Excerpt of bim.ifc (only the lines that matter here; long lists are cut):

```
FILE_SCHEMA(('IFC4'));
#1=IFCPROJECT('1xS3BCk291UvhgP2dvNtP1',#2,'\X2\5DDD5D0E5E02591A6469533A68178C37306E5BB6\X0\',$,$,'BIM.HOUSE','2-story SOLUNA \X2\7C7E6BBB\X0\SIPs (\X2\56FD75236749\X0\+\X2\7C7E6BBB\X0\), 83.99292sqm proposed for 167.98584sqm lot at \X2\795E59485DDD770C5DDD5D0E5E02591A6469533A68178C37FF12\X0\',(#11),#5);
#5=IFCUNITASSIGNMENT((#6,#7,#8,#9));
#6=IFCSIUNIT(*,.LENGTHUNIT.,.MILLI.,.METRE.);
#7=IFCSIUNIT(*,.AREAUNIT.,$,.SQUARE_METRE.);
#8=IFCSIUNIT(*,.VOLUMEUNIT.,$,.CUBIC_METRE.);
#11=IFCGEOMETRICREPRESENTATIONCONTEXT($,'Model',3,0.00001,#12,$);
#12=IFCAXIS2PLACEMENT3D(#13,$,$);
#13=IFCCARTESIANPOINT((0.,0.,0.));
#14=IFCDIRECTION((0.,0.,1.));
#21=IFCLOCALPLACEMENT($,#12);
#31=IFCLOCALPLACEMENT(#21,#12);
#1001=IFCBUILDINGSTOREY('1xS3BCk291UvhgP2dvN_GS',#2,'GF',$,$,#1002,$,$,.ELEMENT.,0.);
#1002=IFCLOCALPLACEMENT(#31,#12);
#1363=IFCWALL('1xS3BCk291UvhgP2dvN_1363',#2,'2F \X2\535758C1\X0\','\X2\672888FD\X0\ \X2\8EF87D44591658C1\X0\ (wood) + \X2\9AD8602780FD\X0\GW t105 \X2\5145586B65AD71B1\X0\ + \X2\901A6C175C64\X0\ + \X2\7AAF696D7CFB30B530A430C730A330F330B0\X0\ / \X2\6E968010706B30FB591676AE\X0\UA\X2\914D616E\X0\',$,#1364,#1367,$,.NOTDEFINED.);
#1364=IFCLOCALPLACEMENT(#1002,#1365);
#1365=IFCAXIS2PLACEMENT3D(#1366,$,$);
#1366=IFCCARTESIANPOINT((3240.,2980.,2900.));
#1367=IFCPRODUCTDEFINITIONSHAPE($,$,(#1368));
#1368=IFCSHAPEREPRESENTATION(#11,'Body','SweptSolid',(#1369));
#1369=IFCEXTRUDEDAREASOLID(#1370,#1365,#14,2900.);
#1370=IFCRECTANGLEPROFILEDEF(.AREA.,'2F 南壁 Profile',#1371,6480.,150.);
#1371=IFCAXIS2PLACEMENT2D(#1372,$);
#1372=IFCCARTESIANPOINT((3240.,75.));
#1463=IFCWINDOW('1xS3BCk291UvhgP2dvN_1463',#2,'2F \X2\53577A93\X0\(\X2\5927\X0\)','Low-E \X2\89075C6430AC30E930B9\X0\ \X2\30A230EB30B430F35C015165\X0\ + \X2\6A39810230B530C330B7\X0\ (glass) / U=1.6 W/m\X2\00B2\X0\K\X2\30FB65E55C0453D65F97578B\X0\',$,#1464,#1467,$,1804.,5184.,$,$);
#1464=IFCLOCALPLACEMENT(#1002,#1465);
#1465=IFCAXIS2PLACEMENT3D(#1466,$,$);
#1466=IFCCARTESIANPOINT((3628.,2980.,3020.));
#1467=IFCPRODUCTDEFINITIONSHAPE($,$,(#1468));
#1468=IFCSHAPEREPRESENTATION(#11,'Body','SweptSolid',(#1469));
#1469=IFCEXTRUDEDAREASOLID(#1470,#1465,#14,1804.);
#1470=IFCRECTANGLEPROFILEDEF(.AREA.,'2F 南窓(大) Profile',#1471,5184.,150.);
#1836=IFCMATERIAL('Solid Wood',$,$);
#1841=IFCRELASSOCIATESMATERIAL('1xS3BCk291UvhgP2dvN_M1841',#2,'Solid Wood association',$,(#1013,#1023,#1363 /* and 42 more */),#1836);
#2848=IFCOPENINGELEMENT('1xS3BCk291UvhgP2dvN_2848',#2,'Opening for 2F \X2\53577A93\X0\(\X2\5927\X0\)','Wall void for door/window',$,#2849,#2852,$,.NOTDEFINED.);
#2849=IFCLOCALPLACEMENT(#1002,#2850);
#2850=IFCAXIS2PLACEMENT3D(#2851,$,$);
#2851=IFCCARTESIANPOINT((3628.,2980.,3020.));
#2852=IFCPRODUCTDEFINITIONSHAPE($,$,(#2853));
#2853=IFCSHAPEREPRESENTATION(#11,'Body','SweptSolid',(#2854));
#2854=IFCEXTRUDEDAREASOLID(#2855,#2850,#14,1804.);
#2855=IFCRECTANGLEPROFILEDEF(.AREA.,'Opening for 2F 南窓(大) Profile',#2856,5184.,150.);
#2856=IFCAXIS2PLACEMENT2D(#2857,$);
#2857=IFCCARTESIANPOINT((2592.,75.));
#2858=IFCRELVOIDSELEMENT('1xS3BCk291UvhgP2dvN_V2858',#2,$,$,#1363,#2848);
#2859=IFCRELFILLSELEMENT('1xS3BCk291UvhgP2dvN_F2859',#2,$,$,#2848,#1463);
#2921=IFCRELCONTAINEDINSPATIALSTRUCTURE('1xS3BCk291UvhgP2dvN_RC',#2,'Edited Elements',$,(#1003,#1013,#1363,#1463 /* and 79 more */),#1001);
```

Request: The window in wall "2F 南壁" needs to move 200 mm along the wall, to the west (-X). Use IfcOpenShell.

```python
import ifcopenshell
import ifcopenshell.api.geometry
import ifcopenshell.util.placement

model = ifcopenshell.open("bim.ifc")

window = model.by_guid("1xS3BCk291UvhgP2dvN_1463")
opening = window.FillsVoids[0].RelatingOpeningElement
wall = opening.VoidsElements[0].RelatingBuildingElement

wall_matrix = ifcopenshell.util.placement.get_local_placement(wall.ObjectPlacement)
shift = wall_matrix[:3, 0] * -200.0
before = ifcopenshell.util.placement.get_local_placement(window.ObjectPlacement)[:3, 3].copy()

# The window is not placed relative to its opening, so move both.
for product in (opening, window):
    matrix = ifcopenshell.util.placement.get_local_placement(product.ObjectPlacement)
    matrix[:3, 3] += shift
    ifcopenshell.api.geometry.edit_object_placement(model, product=product, matrix=matrix, is_si=False)

after = ifcopenshell.util.placement.get_local_placement(window.ObjectPlacement)[:3, 3]
print("window moved by", (after - before).round(3) + 0.0)

model.write("bim_v2.ifc")
```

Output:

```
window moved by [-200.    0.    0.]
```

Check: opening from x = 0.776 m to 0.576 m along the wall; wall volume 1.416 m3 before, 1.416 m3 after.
